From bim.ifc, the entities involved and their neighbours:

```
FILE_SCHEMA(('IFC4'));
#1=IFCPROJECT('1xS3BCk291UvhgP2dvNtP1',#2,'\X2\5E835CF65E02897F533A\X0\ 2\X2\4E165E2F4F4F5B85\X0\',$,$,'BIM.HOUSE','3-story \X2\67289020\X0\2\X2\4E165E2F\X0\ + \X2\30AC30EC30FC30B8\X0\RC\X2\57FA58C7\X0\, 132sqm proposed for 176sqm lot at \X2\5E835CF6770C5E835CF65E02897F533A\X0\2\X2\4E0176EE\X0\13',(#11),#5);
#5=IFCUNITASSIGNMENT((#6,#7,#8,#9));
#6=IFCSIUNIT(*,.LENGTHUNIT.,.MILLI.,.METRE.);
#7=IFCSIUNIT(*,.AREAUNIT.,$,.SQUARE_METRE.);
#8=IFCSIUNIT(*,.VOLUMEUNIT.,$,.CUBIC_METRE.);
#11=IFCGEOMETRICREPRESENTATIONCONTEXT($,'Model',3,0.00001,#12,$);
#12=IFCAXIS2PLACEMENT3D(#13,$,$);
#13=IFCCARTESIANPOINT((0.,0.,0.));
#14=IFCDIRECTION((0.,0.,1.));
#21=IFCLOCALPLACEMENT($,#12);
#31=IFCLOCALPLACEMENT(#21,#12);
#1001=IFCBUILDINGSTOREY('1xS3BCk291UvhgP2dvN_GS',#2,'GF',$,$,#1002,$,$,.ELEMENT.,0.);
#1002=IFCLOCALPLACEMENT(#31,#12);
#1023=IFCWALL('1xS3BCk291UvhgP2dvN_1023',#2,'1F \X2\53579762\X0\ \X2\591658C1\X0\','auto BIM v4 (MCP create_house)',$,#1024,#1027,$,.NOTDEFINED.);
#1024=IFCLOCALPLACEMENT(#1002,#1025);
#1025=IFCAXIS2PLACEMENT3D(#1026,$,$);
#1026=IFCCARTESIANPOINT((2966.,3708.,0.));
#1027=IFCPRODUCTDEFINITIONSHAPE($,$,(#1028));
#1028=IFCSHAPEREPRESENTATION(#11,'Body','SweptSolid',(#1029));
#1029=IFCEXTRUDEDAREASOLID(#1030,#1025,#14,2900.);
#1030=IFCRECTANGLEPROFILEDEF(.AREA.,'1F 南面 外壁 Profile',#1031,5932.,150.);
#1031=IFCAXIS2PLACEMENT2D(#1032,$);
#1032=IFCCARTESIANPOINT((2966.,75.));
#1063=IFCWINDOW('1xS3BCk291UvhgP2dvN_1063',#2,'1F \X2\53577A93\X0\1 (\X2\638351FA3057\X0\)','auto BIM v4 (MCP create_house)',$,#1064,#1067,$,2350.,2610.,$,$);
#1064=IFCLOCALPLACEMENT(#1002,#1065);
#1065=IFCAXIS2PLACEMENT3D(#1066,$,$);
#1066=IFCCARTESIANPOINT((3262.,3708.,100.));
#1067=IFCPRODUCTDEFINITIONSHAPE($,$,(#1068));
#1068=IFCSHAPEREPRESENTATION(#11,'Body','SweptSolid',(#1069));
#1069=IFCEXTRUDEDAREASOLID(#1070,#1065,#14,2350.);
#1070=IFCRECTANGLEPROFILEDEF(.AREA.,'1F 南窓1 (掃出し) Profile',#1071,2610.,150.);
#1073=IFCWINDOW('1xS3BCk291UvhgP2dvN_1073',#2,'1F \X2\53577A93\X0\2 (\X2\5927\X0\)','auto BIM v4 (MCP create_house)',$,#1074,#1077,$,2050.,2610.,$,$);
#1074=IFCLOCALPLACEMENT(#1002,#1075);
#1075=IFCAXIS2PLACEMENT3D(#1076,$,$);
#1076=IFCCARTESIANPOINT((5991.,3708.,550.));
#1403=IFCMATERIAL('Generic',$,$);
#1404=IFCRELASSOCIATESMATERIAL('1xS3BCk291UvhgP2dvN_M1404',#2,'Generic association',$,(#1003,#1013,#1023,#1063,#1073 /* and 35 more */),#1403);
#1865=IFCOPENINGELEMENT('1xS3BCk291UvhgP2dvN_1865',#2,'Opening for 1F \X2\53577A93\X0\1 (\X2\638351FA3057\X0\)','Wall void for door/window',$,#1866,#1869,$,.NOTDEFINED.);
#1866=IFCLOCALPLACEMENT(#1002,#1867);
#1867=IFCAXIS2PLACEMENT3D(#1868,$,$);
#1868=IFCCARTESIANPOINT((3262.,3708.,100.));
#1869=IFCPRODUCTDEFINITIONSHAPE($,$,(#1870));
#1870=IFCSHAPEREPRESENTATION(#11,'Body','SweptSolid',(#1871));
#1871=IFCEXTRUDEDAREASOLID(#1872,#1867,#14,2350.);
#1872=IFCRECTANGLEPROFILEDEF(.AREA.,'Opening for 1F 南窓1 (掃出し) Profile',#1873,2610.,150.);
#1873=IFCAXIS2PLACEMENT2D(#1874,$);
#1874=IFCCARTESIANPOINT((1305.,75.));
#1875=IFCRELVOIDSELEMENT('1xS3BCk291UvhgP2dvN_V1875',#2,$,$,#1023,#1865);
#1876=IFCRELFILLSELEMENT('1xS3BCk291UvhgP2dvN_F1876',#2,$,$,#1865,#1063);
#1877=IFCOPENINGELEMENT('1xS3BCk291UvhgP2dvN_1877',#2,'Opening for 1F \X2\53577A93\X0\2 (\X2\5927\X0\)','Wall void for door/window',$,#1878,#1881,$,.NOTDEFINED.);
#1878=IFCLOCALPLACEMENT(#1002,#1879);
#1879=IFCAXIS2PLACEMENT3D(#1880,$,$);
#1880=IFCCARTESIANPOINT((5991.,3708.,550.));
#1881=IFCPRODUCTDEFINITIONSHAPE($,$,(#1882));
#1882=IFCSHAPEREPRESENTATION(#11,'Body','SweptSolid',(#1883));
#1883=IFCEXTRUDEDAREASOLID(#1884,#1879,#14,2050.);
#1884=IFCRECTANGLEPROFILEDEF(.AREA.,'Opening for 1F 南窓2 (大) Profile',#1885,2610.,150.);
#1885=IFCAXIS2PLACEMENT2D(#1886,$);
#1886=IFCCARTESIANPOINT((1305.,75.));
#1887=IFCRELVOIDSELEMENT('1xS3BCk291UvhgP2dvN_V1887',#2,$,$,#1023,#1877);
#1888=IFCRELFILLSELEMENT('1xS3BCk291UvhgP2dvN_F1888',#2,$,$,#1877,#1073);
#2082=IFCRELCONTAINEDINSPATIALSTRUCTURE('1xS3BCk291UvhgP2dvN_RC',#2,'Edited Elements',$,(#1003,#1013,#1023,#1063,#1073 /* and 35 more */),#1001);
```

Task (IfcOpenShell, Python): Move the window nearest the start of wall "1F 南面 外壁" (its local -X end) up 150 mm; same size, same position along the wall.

```python
import numpy as np
import ifcopenshell
import ifcopenshell.api.geometry
import ifcopenshell.util.placement
import ifcopenshell.util.unit

model = ifcopenshell.open("bim.ifc")
unit_scale = ifcopenshell.util.unit.calculate_unit_scale(model)

window = model.by_guid("1xS3BCk291UvhgP2dvN_1063")
opening = window.FillsVoids[0].RelatingOpeningElement
dz = 0.15 / unit_scale

shift = np.array([0.0, 0.0, dz])
# The window is not placed relative to its opening, so move both.
for product in (opening, window):
    matrix = ifcopenshell.util.placement.get_local_placement(product.ObjectPlacement)
    matrix[:3, 3] += shift
    ifcopenshell.api.geometry.edit_object_placement(model, product=product, matrix=matrix, is_si=False)

print(f"moved by {dz * unit_scale:+.3f} m")

model.write("bim_updated.ifc")
```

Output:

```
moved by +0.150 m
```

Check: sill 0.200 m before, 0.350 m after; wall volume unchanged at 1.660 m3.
